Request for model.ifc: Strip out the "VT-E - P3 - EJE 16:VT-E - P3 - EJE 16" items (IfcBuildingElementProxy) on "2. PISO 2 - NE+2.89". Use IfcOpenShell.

First a look at what the model holds.

```python
import ifcopenshell
import ifcopenshell.util.element

model = ifcopenshell.open("model.ifc")
print(model.schema)
storey = next(s for s in model.by_type("IfcBuildingStorey") if s.Name == "2. PISO 2 - NE+2.89")
proxies = [e for e in ifcopenshell.util.element.get_decomposition(storey) if e.is_a("IfcBuildingElementProxy")]
seen = {}
for e in proxies:
    element_type = ifcopenshell.util.element.get_type(e)
    name = element_type.Name if element_type not in (None, e) else None
    seen[name] = seen.get(name, 0) + 1
for name, count in sorted(seen.items(), key=str):
    print(count, "x", name)
```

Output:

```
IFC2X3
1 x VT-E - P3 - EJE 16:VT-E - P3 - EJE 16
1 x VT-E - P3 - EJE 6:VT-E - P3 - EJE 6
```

```python
import ifcopenshell
import ifcopenshell.api.root
import ifcopenshell.util.element

model = ifcopenshell.open("model.ifc")

storey = next(s for s in model.by_type("IfcBuildingStorey") if s.Name == "2. PISO 2 - NE+2.89")
proxies = [e for e in ifcopenshell.util.element.get_decomposition(storey) if e.is_a("IfcBuildingElementProxy")]
targets = [e for e in proxies if (t := ifcopenshell.util.element.get_type(e)) not in (None, e) and t.Name == "VT-E - P3 - EJE 16:VT-E - P3 - EJE 16"]

for e in targets:
    ifcopenshell.api.root.remove_product(model, product=e)
print(len(targets), "removed")

model.write("model_edited.ifc")
```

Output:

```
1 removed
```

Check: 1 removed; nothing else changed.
